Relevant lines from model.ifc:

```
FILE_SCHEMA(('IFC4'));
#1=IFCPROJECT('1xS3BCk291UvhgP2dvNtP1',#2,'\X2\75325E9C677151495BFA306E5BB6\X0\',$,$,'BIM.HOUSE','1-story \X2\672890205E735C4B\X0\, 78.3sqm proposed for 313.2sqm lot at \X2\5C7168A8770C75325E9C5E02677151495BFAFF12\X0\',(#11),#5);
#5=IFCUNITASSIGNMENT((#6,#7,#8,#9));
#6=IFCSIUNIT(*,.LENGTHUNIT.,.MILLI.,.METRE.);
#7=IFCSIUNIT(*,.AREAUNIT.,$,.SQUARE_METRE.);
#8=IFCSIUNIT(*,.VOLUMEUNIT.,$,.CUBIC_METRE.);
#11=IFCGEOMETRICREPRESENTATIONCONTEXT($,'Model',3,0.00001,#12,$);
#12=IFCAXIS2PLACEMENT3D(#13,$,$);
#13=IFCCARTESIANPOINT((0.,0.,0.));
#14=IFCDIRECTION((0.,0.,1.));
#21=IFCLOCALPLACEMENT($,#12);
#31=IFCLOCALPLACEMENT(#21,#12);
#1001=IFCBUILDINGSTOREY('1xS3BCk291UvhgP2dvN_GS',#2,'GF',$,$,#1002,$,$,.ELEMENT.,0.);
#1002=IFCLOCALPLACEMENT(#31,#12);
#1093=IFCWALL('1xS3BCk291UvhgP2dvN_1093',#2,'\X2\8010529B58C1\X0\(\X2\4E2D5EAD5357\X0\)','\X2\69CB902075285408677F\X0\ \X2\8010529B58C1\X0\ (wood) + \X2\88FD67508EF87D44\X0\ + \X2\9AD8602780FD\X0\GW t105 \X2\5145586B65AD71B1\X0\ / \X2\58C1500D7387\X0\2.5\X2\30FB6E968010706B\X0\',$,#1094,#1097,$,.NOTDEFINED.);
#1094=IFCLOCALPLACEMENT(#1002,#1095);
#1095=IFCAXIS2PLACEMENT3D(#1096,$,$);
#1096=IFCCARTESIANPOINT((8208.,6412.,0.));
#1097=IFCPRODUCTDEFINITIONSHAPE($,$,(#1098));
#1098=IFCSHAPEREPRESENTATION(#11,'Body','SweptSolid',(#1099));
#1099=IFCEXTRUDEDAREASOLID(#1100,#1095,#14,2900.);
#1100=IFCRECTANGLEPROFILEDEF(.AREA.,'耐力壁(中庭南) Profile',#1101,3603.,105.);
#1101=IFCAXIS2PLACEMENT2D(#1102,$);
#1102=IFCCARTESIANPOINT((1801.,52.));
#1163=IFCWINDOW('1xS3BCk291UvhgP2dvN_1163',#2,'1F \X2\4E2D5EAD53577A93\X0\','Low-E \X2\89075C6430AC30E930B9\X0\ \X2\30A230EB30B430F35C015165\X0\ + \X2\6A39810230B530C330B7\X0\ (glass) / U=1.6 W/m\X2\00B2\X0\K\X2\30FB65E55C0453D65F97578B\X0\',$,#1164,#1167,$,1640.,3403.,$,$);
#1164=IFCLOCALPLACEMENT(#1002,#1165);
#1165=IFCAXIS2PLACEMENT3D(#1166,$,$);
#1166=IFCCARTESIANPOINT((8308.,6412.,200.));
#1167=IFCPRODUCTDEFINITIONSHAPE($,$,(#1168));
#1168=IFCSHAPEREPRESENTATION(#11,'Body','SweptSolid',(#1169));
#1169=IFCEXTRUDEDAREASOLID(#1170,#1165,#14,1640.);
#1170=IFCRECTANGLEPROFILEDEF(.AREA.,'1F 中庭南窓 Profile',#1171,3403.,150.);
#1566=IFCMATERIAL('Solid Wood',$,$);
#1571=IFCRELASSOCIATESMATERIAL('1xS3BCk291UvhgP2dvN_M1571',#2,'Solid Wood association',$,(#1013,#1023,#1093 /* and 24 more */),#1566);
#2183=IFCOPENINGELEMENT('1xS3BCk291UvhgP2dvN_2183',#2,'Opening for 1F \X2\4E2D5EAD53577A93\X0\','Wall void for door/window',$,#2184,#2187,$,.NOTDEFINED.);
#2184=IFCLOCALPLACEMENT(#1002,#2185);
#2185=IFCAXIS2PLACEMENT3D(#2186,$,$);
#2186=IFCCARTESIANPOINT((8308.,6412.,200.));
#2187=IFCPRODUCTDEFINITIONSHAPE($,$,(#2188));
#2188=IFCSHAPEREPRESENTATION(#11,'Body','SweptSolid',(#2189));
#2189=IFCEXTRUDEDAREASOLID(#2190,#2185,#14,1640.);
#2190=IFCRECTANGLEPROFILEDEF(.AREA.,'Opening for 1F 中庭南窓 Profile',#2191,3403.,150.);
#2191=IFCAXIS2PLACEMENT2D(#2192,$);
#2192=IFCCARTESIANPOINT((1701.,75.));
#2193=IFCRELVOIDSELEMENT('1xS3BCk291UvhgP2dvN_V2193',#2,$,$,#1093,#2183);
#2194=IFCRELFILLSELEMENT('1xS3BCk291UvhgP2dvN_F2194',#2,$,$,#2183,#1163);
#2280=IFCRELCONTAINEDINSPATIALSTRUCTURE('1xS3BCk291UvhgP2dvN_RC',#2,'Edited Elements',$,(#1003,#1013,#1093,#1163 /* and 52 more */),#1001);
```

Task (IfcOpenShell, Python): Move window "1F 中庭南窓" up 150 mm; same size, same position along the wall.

```python
import numpy as np
import ifcopenshell
import ifcopenshell.api.geometry
import ifcopenshell.util.placement
import ifcopenshell.util.unit

model = ifcopenshell.open("model.ifc")
unit_scale = ifcopenshell.util.unit.calculate_unit_scale(model)

window = model.by_guid("1xS3BCk291UvhgP2dvN_1163")
opening = window.FillsVoids[0].RelatingOpeningElement
dz = 150.0

shift = np.array([0.0, 0.0, dz])
# The window is not placed relative to its opening, so move both.
for product in (opening, window):
    matrix = ifcopenshell.util.placement.get_local_placement(product.ObjectPlacement)
    matrix[:3, 3] += shift
    ifcopenshell.api.geometry.edit_object_placement(model, product=product, matrix=matrix, is_si=False)

print(f"moved by {dz * unit_scale:+.3f} m")

model.write("model_updated.ifc")
```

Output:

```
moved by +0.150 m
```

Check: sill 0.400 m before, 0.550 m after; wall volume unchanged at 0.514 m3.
